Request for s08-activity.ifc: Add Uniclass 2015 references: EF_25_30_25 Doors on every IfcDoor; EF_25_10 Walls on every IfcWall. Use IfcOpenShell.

First a look at what the model holds.

```python
import ifcopenshell

model = ifcopenshell.open("s08-activity.ifc")
print(model.schema)
print("classifications:", [c.Name for c in model.by_type("IfcClassification")])
for ifc_class in ("IfcDoor", "IfcRoof", "IfcStair", "IfcWall", "IfcWindow"):
    print(ifc_class, len(model.by_type(ifc_class)))
```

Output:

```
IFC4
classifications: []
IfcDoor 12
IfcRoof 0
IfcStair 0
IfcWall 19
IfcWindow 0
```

```python
import ifcopenshell
import ifcopenshell.api.classification

model = ifcopenshell.open("s08-activity.ifc")

system = ifcopenshell.api.classification.add_classification(model, classification="Uniclass 2015")

codes = {
    "IfcDoor": ("EF_25_30_25", "Doors"),
    "IfcWall": ("EF_25_10", "Walls"),
}
for ifc_class, (code, name) in codes.items():
    products = model.by_type(ifc_class)
    ifcopenshell.api.classification.add_reference(
        model, products=products, classification=system, identification=code, name=name
    )
    print(code, len(products))

model.write("s08-activity-out.ifc")
```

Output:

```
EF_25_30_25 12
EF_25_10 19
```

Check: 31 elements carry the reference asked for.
